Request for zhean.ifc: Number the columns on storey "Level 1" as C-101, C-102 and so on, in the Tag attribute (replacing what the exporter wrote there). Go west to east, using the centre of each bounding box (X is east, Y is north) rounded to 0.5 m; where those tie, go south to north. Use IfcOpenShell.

First a look at what the model holds.

```python
import ifcopenshell
import ifcopenshell.util.element
import ifcopenshell.util.placement

model = ifcopenshell.open("zhean.ifc")
print(model.schema)
storey = next(s for s in model.by_type("IfcBuildingStorey") if s.Name == "Level 1")
columns = [e for e in ifcopenshell.util.element.get_decomposition(storey) if e.is_a("IfcColumn")]
for e in sorted(columns, key=lambda e: e.id()):
    origin = ifcopenshell.util.placement.get_local_placement(e.ObjectPlacement)[:3, 3]
    print(e.id(), e.Tag, e.Name, origin.round(2) + 0.0, sep=" | ")
```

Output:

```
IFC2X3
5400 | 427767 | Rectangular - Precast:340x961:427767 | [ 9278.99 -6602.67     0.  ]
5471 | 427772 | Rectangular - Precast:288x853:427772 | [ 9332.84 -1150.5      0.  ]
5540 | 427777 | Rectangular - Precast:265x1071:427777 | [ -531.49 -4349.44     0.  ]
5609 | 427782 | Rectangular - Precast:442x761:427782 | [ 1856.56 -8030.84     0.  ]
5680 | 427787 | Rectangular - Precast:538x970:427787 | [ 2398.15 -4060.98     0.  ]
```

```python
import ifcopenshell
import ifcopenshell.geom
import ifcopenshell.util.element
import ifcopenshell.util.shape

model = ifcopenshell.open("zhean.ifc")
settings = ifcopenshell.geom.settings()
settings.set("use-world-coords", True)


def centre(element):
    shape = ifcopenshell.geom.create_shape(settings, element)
    return ifcopenshell.util.shape.get_bbox_centroid(shape.geometry)


storey = next(s for s in model.by_type("IfcBuildingStorey") if s.Name == "Level 1")
columns = [e for e in ifcopenshell.util.element.get_decomposition(storey) if e.is_a("IfcColumn")]

# Insertion points can sit at a corner or the storey origin, so sort by the geometry (in metres).
centres = {e: centre(e) for e in columns}
columns.sort(key=lambda e: (round(centres[e][0] / 0.5), centres[e][1]))

for i, e in enumerate(columns, start=1):
    number = f"C-1{i:02d}"
    e.Tag = number
    print(e.id(), number)

model.write("zhean-out.ifc")
```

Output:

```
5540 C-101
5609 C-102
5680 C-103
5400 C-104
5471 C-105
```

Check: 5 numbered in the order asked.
